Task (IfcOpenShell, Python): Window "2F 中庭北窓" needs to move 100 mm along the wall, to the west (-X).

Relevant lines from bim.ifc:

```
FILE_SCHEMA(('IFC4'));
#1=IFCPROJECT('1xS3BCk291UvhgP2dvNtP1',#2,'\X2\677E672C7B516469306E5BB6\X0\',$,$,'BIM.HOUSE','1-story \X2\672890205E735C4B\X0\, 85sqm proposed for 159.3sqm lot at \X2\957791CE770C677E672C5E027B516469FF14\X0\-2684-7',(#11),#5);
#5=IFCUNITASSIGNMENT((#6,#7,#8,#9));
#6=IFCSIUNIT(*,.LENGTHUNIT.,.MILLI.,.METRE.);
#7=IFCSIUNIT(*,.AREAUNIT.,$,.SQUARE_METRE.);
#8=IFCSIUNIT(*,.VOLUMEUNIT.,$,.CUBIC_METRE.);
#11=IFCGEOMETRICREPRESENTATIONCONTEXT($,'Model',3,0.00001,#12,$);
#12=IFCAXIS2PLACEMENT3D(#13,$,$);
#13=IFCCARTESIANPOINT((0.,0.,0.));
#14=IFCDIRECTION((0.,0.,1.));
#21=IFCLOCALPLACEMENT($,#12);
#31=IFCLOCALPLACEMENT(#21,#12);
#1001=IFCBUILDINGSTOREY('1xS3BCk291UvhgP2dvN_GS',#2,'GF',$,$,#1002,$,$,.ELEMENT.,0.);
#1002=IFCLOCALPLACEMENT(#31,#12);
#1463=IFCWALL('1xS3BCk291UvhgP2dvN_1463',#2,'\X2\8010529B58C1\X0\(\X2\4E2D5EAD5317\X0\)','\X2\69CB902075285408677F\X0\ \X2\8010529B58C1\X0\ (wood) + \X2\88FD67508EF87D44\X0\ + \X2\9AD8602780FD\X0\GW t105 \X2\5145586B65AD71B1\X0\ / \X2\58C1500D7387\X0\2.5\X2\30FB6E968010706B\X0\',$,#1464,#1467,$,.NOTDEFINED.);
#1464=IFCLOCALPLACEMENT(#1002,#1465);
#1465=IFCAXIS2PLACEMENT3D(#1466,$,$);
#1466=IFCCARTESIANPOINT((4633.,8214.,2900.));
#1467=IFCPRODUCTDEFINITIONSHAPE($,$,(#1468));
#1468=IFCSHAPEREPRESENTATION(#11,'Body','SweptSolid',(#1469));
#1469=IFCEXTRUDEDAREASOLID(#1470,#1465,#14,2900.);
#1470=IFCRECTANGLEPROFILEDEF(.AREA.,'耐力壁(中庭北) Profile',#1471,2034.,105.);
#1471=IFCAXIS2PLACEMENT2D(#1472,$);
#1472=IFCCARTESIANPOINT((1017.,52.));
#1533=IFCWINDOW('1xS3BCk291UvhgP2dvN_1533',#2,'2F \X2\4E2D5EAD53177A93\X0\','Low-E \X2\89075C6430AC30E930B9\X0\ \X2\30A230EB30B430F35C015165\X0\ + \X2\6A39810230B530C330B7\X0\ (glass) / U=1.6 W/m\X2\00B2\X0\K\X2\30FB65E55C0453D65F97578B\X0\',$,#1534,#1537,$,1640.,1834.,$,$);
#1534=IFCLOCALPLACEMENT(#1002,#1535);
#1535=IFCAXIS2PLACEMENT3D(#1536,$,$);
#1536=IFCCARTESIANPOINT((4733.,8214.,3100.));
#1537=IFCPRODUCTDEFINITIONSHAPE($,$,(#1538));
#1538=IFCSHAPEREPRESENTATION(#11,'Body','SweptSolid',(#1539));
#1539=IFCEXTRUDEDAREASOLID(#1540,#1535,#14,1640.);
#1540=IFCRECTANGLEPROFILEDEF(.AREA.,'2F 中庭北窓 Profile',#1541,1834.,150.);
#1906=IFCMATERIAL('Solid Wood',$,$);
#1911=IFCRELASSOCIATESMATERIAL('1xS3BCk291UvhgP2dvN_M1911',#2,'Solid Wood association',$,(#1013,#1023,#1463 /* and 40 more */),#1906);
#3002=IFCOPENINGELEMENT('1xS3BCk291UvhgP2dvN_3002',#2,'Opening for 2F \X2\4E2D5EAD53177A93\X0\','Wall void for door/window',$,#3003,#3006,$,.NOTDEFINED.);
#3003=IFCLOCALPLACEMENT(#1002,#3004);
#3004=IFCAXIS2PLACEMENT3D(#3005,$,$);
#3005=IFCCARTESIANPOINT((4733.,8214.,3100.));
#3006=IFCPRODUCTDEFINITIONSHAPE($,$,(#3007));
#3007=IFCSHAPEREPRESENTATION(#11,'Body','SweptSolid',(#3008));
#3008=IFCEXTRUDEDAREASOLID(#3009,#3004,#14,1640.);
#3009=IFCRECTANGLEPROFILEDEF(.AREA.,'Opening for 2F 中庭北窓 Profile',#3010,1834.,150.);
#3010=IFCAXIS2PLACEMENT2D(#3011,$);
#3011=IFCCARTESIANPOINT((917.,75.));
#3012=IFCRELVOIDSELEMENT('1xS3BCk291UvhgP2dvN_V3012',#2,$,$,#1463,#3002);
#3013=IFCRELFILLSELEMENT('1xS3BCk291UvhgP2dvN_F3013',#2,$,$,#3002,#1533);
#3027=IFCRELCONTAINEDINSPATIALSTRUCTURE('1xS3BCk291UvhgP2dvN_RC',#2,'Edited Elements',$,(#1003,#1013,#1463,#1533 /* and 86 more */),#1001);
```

```python
import ifcopenshell
import ifcopenshell.api.geometry
import ifcopenshell.util.placement
import ifcopenshell.util.unit

model = ifcopenshell.open("bim.ifc")
unit_scale = ifcopenshell.util.unit.calculate_unit_scale(model)

window = model.by_guid("1xS3BCk291UvhgP2dvN_1533")
opening = window.FillsVoids[0].RelatingOpeningElement
wall = opening.VoidsElements[0].RelatingBuildingElement

wall_matrix = ifcopenshell.util.placement.get_local_placement(wall.ObjectPlacement)
shift = wall_matrix[:3, 0] * -0.1 / unit_scale
before = ifcopenshell.util.placement.get_local_placement(window.ObjectPlacement)[:3, 3].copy()

# The window is not placed relative to its opening, so move both.
for product in (opening, window):
    matrix = ifcopenshell.util.placement.get_local_placement(product.ObjectPlacement)
    matrix[:3, 3] += shift
    ifcopenshell.api.geometry.edit_object_placement(model, product=product, matrix=matrix, is_si=False)

after = ifcopenshell.util.placement.get_local_placement(window.ObjectPlacement)[:3, 3]
print("window moved by", (after - before).round(3) + 0.0)

model.write("bim-out.ifc")
```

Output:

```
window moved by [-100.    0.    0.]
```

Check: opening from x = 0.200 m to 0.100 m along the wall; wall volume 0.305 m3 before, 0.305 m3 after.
